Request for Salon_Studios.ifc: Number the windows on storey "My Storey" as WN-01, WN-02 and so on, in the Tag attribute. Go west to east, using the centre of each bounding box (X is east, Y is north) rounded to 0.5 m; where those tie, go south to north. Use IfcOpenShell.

First a look at what the model holds.

```python
import ifcopenshell
import ifcopenshell.util.element
import ifcopenshell.util.placement

model = ifcopenshell.open("Salon_Studios.ifc")
print(model.schema)
storey = next(s for s in model.by_type("IfcBuildingStorey") if s.Name == "My Storey")
windows = [e for e in ifcopenshell.util.element.get_decomposition(storey) if e.is_a("IfcWindow")]
for e in sorted(windows, key=lambda e: e.id()):
    origin = ifcopenshell.util.placement.get_local_placement(e.ObjectPlacement)[:3, 3]
    print(e.id(), e.Tag, e.Name, origin.round(2) + 0.0, sep=" | ")
```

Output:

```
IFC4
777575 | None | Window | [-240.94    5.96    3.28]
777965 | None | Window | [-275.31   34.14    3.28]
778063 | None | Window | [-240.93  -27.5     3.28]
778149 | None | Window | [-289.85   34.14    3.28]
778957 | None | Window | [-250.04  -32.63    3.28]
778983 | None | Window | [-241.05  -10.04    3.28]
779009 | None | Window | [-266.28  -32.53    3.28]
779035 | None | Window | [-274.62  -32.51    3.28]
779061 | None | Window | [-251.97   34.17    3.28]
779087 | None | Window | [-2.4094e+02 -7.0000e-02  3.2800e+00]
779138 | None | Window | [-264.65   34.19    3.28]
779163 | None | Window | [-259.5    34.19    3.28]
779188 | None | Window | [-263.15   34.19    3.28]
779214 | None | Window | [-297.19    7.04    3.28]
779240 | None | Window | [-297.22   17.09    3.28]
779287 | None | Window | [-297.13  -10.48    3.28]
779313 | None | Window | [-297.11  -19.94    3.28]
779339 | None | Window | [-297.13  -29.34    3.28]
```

```python
import ifcopenshell
import ifcopenshell.geom
import ifcopenshell.util.element
import ifcopenshell.util.shape

model = ifcopenshell.open("Salon_Studios.ifc")
settings = ifcopenshell.geom.settings()
settings.set("use-world-coords", True)


def centre(element):
    shape = ifcopenshell.geom.create_shape(settings, element)
    return ifcopenshell.util.shape.get_bbox_centroid(shape.geometry)


storey = next(s for s in model.by_type("IfcBuildingStorey") if s.Name == "My Storey")
windows = [e for e in ifcopenshell.util.element.get_decomposition(storey) if e.is_a("IfcWindow")]

# Insertion points can sit at a corner or the storey origin, so sort by the geometry (in metres).
centres = {e: centre(e) for e in windows}
windows.sort(key=lambda e: (round(centres[e][0] / 0.5), centres[e][1]))

for i, e in enumerate(windows, start=1):
    number = f"WN-{i:02d}"
    e.Tag = number
    print(e.id(), number)

model.write("Salon_Studios_v2.ifc")
```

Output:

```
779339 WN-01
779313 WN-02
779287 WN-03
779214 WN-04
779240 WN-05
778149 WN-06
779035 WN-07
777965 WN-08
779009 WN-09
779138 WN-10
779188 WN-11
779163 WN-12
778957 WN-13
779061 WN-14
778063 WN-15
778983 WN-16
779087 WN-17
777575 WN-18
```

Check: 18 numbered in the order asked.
